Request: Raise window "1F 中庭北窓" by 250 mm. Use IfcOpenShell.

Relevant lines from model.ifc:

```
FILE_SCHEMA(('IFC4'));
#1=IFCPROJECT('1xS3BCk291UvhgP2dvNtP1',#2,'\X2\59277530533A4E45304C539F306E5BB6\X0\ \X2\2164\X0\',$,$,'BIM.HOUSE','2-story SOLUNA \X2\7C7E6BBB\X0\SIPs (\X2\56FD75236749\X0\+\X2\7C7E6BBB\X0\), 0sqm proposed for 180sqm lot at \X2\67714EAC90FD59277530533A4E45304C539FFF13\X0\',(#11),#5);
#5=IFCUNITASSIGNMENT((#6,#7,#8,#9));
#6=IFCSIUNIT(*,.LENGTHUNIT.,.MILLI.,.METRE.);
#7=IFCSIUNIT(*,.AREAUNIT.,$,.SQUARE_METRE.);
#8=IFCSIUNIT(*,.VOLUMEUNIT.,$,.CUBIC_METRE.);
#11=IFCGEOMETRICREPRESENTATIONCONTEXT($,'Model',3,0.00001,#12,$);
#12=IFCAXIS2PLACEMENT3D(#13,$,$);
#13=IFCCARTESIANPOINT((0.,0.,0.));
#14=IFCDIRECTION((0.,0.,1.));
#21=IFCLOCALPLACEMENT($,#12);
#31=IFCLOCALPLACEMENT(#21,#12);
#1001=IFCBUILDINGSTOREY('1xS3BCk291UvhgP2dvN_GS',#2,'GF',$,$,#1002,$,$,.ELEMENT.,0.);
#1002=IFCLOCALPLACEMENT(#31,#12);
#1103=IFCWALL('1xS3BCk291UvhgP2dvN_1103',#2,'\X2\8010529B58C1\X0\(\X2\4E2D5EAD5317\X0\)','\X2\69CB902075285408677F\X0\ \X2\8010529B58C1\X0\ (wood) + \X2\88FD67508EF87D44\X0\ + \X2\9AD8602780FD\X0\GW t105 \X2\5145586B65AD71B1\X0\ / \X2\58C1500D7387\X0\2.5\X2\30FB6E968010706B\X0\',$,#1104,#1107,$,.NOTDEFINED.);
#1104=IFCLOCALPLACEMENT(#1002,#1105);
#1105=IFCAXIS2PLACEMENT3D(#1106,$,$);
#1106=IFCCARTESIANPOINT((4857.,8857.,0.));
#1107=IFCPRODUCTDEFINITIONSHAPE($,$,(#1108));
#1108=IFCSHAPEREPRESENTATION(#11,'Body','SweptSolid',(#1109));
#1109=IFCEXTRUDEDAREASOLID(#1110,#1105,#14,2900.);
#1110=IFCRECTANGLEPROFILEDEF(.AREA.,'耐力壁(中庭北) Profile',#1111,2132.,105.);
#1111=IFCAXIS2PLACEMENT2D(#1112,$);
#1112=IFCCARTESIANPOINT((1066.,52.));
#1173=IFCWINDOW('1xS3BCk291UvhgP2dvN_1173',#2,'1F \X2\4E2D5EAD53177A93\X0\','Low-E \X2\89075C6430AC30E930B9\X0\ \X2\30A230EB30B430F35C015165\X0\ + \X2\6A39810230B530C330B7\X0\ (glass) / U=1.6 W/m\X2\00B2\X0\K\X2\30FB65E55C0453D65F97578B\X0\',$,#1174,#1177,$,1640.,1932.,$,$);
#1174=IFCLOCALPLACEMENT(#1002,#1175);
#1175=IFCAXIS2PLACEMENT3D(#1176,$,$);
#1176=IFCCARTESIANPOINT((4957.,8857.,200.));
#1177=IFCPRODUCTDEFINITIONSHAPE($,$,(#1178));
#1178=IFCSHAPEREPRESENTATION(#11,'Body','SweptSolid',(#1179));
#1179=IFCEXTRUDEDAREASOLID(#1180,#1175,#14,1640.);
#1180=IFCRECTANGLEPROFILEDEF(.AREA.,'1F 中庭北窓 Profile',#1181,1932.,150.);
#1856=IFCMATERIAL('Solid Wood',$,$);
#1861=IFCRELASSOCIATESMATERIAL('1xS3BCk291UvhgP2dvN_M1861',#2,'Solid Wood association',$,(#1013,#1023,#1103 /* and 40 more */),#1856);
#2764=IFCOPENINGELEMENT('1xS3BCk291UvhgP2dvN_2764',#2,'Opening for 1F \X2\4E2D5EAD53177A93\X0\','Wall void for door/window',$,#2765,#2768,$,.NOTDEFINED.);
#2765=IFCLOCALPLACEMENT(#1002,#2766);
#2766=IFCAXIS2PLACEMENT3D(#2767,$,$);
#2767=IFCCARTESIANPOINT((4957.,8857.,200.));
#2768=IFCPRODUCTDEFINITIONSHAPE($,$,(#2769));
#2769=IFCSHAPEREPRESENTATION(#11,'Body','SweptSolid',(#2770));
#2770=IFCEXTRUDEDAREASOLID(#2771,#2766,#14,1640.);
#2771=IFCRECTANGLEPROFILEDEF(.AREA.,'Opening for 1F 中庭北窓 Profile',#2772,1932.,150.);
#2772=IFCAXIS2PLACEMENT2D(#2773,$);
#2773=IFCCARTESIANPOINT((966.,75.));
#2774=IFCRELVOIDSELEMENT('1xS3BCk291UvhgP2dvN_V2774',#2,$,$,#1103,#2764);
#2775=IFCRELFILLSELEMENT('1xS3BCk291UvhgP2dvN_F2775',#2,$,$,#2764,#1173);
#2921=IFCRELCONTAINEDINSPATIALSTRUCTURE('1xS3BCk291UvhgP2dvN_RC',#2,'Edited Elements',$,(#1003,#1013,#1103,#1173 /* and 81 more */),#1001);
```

```python
import numpy as np
import ifcopenshell
import ifcopenshell.api.geometry
import ifcopenshell.util.placement
import ifcopenshell.util.unit

model = ifcopenshell.open("model.ifc")
unit_scale = ifcopenshell.util.unit.calculate_unit_scale(model)

window = model.by_guid("1xS3BCk291UvhgP2dvN_1173")
opening = window.FillsVoids[0].RelatingOpeningElement
dz = 0.25 / unit_scale

shift = np.array([0.0, 0.0, dz])
# The window is not placed relative to its opening, so move both.
for product in (opening, window):
    matrix = ifcopenshell.util.placement.get_local_placement(product.ObjectPlacement)
    matrix[:3, 3] += shift
    ifcopenshell.api.geometry.edit_object_placement(model, product=product, matrix=matrix, is_si=False)

print(f"moved by {dz * unit_scale:+.3f} m")

model.write("model_rev.ifc")
```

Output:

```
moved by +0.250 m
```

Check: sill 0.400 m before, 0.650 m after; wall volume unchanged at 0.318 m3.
